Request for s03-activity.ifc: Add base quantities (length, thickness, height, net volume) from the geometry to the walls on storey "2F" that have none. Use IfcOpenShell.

First a look at what the model holds.

```python
import ifcopenshell
import ifcopenshell.util.element
import ifcopenshell.util.unit

model = ifcopenshell.open("s03-activity.ifc")
print(model.schema)
for unit_type in ("LENGTHUNIT", "AREAUNIT", "VOLUMEUNIT"):
    print(unit_type, ifcopenshell.util.unit.calculate_unit_scale(model, unit_type))
storey = next(s for s in model.by_type("IfcBuildingStorey") if s.Name == "2F")
walls = [e for e in ifcopenshell.util.element.get_decomposition(storey) if e.is_a("IfcWall")]
for e in sorted(walls, key=lambda e: e.id()):
    print(e.id(), e.is_a(), e.Name, list(ifcopenshell.util.element.get_psets(e, qtos_only=True)), sep=" | ")
```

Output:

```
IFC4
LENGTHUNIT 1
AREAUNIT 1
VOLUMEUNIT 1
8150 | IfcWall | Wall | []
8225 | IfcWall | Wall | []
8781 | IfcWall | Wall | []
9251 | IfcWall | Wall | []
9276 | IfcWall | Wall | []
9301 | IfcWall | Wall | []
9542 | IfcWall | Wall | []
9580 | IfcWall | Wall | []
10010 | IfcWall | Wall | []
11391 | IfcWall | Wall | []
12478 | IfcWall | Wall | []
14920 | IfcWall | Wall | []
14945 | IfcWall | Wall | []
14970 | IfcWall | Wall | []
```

```python
import ifcopenshell
import ifcopenshell.api.pset
import ifcopenshell.geom
import ifcopenshell.util.element
import ifcopenshell.util.shape
import ifcopenshell.util.unit

model = ifcopenshell.open("s03-activity.ifc")
unit_scale = ifcopenshell.util.unit.calculate_unit_scale(model)
volume_scale = ifcopenshell.util.unit.calculate_unit_scale(model, "VOLUMEUNIT")
settings = ifcopenshell.geom.settings()

storey = next(s for s in model.by_type("IfcBuildingStorey") if s.Name == "2F")
walls = [e for e in ifcopenshell.util.element.get_decomposition(storey) if e.is_a("IfcWall")]

for e in sorted(walls, key=lambda e: e.id()):
    if ifcopenshell.util.element.get_psets(e, qtos_only=True, should_inherit=False):
        continue
    # Geometry comes back in metres, in the element's own axes.
    shape = ifcopenshell.geom.create_shape(settings, e)
    values = {
        "Length": ifcopenshell.util.shape.get_x(shape.geometry) / unit_scale,
        "Width": ifcopenshell.util.shape.get_y(shape.geometry) / unit_scale,
        "Height": ifcopenshell.util.shape.get_z(shape.geometry) / unit_scale,
        "NetVolume": ifcopenshell.util.shape.get_volume(shape.geometry) / volume_scale,
    }
    qto = ifcopenshell.api.pset.add_qto(model, product=e, name="Qto_WallBaseQuantities")
    ifcopenshell.api.pset.edit_qto(model, qto=qto, properties=values)
    print(e.id(), {k: round(v, 3) for k, v in values.items()})

model.write("s03-activity_edited.ifc")
```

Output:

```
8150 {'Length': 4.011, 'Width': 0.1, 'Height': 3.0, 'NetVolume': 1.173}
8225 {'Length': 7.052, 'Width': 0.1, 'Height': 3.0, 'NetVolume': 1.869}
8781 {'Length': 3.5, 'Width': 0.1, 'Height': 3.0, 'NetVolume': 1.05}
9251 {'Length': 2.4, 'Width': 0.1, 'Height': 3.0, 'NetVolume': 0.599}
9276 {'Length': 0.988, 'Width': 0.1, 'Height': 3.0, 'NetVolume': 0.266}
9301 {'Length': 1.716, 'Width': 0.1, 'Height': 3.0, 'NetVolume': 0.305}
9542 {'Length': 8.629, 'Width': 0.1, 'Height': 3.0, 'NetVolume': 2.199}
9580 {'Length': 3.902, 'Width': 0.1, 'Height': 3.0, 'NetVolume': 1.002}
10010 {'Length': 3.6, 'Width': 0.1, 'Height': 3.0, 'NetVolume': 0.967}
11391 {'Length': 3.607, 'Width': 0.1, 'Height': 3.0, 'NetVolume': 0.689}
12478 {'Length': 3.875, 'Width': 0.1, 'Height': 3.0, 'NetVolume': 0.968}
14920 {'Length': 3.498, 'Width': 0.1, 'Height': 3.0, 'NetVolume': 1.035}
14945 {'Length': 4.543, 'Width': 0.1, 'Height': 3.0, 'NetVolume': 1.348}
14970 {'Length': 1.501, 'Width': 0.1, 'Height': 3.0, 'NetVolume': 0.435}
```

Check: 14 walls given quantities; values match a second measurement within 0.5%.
